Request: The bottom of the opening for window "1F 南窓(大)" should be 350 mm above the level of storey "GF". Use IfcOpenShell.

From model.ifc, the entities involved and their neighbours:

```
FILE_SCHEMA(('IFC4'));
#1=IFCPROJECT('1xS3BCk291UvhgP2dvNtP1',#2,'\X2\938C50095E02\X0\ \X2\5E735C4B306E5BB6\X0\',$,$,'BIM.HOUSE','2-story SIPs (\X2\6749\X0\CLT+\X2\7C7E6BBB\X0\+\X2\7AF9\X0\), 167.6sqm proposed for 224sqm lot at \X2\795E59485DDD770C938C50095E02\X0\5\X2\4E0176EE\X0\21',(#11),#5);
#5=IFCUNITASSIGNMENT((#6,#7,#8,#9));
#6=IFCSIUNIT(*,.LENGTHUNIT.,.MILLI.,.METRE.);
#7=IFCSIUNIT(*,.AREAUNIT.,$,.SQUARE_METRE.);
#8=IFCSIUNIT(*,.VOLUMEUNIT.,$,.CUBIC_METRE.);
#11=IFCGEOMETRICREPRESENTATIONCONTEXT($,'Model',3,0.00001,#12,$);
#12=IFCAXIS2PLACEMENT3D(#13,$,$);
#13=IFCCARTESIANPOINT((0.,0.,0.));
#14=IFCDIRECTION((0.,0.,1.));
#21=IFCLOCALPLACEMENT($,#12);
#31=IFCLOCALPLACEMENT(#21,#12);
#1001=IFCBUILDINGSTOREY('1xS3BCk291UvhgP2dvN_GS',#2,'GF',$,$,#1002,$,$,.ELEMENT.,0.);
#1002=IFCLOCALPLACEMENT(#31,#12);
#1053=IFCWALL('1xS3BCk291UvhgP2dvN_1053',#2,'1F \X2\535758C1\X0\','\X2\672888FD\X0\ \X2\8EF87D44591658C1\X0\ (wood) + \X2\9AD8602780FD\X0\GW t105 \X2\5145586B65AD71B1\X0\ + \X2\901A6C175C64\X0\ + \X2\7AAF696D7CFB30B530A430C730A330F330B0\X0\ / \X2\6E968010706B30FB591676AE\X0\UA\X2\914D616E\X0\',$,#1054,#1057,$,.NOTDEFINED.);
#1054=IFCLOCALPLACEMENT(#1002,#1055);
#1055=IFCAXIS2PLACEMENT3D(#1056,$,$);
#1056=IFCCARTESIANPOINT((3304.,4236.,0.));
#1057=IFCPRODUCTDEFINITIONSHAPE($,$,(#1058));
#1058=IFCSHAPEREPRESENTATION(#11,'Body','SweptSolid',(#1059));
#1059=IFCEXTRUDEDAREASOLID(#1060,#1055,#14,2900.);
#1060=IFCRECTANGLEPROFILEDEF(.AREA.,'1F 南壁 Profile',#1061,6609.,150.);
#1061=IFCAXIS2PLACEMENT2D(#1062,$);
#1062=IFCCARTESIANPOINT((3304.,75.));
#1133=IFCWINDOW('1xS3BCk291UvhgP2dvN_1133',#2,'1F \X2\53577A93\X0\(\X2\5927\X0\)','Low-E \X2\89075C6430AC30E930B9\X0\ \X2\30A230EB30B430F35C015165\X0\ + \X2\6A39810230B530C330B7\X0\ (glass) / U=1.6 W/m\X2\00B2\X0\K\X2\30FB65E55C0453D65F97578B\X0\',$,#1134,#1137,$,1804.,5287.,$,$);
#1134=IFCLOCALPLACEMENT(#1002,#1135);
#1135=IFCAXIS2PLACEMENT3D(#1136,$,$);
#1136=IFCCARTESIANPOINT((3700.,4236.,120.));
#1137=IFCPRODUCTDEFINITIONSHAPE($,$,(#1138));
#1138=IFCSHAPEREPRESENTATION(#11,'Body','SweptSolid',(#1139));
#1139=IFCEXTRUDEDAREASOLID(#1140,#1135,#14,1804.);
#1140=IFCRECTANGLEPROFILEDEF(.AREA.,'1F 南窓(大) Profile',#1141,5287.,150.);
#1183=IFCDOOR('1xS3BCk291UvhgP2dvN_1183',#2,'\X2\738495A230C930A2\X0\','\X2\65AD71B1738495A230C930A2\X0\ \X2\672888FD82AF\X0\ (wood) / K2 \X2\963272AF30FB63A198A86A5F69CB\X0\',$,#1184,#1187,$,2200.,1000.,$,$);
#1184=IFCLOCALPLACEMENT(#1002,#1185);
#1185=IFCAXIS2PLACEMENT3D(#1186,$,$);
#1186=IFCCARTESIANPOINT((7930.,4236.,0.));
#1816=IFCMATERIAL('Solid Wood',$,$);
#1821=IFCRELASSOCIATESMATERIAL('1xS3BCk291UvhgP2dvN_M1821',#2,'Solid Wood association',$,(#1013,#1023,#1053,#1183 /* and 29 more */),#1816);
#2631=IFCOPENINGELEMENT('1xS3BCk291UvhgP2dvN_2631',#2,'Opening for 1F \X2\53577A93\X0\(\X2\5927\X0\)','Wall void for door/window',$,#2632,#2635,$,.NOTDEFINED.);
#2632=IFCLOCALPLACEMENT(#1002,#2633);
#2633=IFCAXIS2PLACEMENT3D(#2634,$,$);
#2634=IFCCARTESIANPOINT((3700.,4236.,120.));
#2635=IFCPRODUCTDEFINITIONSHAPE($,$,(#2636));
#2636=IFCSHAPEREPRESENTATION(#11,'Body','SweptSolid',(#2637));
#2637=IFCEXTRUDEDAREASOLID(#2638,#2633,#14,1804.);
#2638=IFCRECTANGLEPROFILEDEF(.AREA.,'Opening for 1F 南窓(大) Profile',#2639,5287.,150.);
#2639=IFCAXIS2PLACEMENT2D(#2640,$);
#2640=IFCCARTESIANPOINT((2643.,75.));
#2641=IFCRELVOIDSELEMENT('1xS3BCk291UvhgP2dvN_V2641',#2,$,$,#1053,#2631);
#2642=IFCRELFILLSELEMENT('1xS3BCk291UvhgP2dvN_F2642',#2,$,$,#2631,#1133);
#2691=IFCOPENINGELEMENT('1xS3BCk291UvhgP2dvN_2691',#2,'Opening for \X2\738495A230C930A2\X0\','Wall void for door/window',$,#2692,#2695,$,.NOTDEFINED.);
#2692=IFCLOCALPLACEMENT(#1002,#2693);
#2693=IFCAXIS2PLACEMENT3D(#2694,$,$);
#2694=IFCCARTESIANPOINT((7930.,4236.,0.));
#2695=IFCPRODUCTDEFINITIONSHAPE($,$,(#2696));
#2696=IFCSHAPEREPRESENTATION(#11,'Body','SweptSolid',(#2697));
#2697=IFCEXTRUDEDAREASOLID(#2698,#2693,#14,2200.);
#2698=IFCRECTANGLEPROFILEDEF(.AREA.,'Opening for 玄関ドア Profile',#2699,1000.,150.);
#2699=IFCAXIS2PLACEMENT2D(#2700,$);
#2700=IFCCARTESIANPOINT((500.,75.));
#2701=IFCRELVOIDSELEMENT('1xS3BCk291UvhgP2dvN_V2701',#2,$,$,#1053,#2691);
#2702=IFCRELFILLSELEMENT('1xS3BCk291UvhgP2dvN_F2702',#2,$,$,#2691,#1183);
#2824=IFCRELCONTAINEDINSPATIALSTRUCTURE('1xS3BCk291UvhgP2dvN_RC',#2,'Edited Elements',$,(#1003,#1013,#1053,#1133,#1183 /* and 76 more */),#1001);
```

```python
import numpy as np
import ifcopenshell
import ifcopenshell.api.geometry
import ifcopenshell.geom
import ifcopenshell.util.element
import ifcopenshell.util.placement
import ifcopenshell.util.shape
import ifcopenshell.util.unit

model = ifcopenshell.open("model.ifc")
unit_scale = ifcopenshell.util.unit.calculate_unit_scale(model)

window = model.by_guid("1xS3BCk291UvhgP2dvN_1133")
opening = window.FillsVoids[0].RelatingOpeningElement
storey = ifcopenshell.util.element.get_container(window, ifc_class="IfcBuildingStorey")
level = ifcopenshell.util.placement.get_local_placement(storey.ObjectPlacement)[2, 3]

# The opening's origin need not be at the sill, so measure its lowest point.
shape = ifcopenshell.geom.create_shape(ifcopenshell.geom.settings(), opening)
bottom = ifcopenshell.util.shape.get_shape_bottom_elevation(shape, shape.geometry) / unit_scale
dz = level + 350.0 - bottom

shift = np.array([0.0, 0.0, dz])
# The window is not placed relative to its opening, so move both.
for product in (opening, window):
    matrix = ifcopenshell.util.placement.get_local_placement(product.ObjectPlacement)
    matrix[:3, 3] += shift
    ifcopenshell.api.geometry.edit_object_placement(model, product=product, matrix=matrix, is_si=False)

print(f"moved by {dz * unit_scale:+.3f} m")

model.write("model-out.ifc")
```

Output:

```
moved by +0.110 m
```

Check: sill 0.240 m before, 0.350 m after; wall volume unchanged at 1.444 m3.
